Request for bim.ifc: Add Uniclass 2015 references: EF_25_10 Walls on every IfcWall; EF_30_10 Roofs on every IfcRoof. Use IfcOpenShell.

First a look at what the model holds.

```python
import ifcopenshell

model = ifcopenshell.open("bim.ifc")
print(model.schema)
print("classifications:", [c.Name for c in model.by_type("IfcClassification")])
for ifc_class in ("IfcDoor", "IfcRoof", "IfcStair", "IfcWall", "IfcWindow"):
    print(ifc_class, len(model.by_type(ifc_class)))
```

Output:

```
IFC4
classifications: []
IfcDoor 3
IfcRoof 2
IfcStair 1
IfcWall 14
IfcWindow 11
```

```python
import ifcopenshell
import ifcopenshell.api.classification

model = ifcopenshell.open("bim.ifc")

system = ifcopenshell.api.classification.add_classification(model, classification="Uniclass 2015")

codes = {
    "IfcWall": ("EF_25_10", "Walls"),
    "IfcRoof": ("EF_30_10", "Roofs"),
}
for ifc_class, (code, name) in codes.items():
    products = model.by_type(ifc_class)
    ifcopenshell.api.classification.add_reference(
        model, products=products, classification=system, identification=code, name=name
    )
    print(code, len(products))

model.write("bim-out.ifc")
```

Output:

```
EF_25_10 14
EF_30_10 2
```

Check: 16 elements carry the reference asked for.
